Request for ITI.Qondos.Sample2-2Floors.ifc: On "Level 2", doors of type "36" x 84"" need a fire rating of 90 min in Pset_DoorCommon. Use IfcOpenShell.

First a look at what the model holds.

```python
import ifcopenshell
import ifcopenshell.util.element

model = ifcopenshell.open("ITI.Qondos.Sample2-2Floors.ifc")
print(model.schema)
storey = next(s for s in model.by_type("IfcBuildingStorey") if s.Name == "Level 2")
doors = [e for e in ifcopenshell.util.element.get_decomposition(storey) if e.is_a("IfcDoor")]
seen = {}
for e in doors:
    element_type = ifcopenshell.util.element.get_type(e)
    key = (element_type.Name if element_type != e and element_type else None, ifcopenshell.util.element.get_pset(e, "Pset_DoorCommon", "FireRating"))
    seen[key] = seen.get(key, 0) + 1
for (name, value), count in sorted(seen.items(), key=str):
    print(count, "x", name, "|", value)
```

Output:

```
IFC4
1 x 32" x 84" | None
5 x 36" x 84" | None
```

```python
import ifcopenshell
import ifcopenshell.api.pset
import ifcopenshell.util.element

model = ifcopenshell.open("ITI.Qondos.Sample2-2Floors.ifc")

storey = next(s for s in model.by_type("IfcBuildingStorey") if s.Name == "Level 2")
doors = [e for e in ifcopenshell.util.element.get_decomposition(storey) if e.is_a("IfcDoor")]

count = 0
for e in doors:
    element_type = ifcopenshell.util.element.get_type(e)
    if element_type in (None, e) or element_type.Name != '36" x 84"':
        continue
    # add_pset returns the element's existing set when there is one.
    pset = ifcopenshell.api.pset.add_pset(model, product=e, name="Pset_DoorCommon")
    ifcopenshell.api.pset.edit_pset(model, pset=pset, properties={"FireRating": "90 min"})
    count += 1

print(count, "doors updated")

model.write("ITI.Qondos.Sample2-2Floors_v2.ifc")
```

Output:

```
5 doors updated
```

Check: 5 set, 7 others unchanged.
